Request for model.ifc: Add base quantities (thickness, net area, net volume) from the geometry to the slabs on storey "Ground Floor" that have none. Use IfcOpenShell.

First a look at what the model holds.

```python
import ifcopenshell
import ifcopenshell.util.element
import ifcopenshell.util.unit

model = ifcopenshell.open("model.ifc")
print(model.schema)
for unit_type in ("LENGTHUNIT", "AREAUNIT", "VOLUMEUNIT"):
    print(unit_type, ifcopenshell.util.unit.calculate_unit_scale(model, unit_type))
storey = next(s for s in model.by_type("IfcBuildingStorey") if s.Name == "Ground Floor")
slabs = [e for e in ifcopenshell.util.element.get_decomposition(storey) if e.is_a("IfcSlab")]
for e in sorted(slabs, key=lambda e: e.id()):
    print(e.id(), e.is_a(), e.Name, list(ifcopenshell.util.element.get_psets(e, qtos_only=True)), sep=" | ")
```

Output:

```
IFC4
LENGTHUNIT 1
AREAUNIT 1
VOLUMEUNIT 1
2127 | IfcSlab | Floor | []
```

```python
import ifcopenshell
import ifcopenshell.api.pset
import ifcopenshell.geom
import ifcopenshell.util.element
import ifcopenshell.util.shape
import ifcopenshell.util.unit

model = ifcopenshell.open("model.ifc")
unit_scale = ifcopenshell.util.unit.calculate_unit_scale(model)
area_scale = ifcopenshell.util.unit.calculate_unit_scale(model, "AREAUNIT")
volume_scale = ifcopenshell.util.unit.calculate_unit_scale(model, "VOLUMEUNIT")
settings = ifcopenshell.geom.settings()

storey = next(s for s in model.by_type("IfcBuildingStorey") if s.Name == "Ground Floor")
slabs = [e for e in ifcopenshell.util.element.get_decomposition(storey) if e.is_a("IfcSlab")]

for e in sorted(slabs, key=lambda e: e.id()):
    if ifcopenshell.util.element.get_psets(e, qtos_only=True, should_inherit=False):
        continue
    # Geometry comes back in metres, in the element's own axes.
    shape = ifcopenshell.geom.create_shape(settings, e)
    values = {
        "Width": ifcopenshell.util.shape.get_z(shape.geometry) / unit_scale,
        "NetArea": ifcopenshell.util.shape.get_footprint_area(shape.geometry) / area_scale,
        "NetVolume": ifcopenshell.util.shape.get_volume(shape.geometry) / volume_scale,
    }
    qto = ifcopenshell.api.pset.add_qto(model, product=e, name="Qto_SlabBaseQuantities")
    ifcopenshell.api.pset.edit_qto(model, qto=qto, properties=values)
    print(e.id(), {k: round(v, 3) for k, v in values.items()})

model.write("model_edited.ifc")
```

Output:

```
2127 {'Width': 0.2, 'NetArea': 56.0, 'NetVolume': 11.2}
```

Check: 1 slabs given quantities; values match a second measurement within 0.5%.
